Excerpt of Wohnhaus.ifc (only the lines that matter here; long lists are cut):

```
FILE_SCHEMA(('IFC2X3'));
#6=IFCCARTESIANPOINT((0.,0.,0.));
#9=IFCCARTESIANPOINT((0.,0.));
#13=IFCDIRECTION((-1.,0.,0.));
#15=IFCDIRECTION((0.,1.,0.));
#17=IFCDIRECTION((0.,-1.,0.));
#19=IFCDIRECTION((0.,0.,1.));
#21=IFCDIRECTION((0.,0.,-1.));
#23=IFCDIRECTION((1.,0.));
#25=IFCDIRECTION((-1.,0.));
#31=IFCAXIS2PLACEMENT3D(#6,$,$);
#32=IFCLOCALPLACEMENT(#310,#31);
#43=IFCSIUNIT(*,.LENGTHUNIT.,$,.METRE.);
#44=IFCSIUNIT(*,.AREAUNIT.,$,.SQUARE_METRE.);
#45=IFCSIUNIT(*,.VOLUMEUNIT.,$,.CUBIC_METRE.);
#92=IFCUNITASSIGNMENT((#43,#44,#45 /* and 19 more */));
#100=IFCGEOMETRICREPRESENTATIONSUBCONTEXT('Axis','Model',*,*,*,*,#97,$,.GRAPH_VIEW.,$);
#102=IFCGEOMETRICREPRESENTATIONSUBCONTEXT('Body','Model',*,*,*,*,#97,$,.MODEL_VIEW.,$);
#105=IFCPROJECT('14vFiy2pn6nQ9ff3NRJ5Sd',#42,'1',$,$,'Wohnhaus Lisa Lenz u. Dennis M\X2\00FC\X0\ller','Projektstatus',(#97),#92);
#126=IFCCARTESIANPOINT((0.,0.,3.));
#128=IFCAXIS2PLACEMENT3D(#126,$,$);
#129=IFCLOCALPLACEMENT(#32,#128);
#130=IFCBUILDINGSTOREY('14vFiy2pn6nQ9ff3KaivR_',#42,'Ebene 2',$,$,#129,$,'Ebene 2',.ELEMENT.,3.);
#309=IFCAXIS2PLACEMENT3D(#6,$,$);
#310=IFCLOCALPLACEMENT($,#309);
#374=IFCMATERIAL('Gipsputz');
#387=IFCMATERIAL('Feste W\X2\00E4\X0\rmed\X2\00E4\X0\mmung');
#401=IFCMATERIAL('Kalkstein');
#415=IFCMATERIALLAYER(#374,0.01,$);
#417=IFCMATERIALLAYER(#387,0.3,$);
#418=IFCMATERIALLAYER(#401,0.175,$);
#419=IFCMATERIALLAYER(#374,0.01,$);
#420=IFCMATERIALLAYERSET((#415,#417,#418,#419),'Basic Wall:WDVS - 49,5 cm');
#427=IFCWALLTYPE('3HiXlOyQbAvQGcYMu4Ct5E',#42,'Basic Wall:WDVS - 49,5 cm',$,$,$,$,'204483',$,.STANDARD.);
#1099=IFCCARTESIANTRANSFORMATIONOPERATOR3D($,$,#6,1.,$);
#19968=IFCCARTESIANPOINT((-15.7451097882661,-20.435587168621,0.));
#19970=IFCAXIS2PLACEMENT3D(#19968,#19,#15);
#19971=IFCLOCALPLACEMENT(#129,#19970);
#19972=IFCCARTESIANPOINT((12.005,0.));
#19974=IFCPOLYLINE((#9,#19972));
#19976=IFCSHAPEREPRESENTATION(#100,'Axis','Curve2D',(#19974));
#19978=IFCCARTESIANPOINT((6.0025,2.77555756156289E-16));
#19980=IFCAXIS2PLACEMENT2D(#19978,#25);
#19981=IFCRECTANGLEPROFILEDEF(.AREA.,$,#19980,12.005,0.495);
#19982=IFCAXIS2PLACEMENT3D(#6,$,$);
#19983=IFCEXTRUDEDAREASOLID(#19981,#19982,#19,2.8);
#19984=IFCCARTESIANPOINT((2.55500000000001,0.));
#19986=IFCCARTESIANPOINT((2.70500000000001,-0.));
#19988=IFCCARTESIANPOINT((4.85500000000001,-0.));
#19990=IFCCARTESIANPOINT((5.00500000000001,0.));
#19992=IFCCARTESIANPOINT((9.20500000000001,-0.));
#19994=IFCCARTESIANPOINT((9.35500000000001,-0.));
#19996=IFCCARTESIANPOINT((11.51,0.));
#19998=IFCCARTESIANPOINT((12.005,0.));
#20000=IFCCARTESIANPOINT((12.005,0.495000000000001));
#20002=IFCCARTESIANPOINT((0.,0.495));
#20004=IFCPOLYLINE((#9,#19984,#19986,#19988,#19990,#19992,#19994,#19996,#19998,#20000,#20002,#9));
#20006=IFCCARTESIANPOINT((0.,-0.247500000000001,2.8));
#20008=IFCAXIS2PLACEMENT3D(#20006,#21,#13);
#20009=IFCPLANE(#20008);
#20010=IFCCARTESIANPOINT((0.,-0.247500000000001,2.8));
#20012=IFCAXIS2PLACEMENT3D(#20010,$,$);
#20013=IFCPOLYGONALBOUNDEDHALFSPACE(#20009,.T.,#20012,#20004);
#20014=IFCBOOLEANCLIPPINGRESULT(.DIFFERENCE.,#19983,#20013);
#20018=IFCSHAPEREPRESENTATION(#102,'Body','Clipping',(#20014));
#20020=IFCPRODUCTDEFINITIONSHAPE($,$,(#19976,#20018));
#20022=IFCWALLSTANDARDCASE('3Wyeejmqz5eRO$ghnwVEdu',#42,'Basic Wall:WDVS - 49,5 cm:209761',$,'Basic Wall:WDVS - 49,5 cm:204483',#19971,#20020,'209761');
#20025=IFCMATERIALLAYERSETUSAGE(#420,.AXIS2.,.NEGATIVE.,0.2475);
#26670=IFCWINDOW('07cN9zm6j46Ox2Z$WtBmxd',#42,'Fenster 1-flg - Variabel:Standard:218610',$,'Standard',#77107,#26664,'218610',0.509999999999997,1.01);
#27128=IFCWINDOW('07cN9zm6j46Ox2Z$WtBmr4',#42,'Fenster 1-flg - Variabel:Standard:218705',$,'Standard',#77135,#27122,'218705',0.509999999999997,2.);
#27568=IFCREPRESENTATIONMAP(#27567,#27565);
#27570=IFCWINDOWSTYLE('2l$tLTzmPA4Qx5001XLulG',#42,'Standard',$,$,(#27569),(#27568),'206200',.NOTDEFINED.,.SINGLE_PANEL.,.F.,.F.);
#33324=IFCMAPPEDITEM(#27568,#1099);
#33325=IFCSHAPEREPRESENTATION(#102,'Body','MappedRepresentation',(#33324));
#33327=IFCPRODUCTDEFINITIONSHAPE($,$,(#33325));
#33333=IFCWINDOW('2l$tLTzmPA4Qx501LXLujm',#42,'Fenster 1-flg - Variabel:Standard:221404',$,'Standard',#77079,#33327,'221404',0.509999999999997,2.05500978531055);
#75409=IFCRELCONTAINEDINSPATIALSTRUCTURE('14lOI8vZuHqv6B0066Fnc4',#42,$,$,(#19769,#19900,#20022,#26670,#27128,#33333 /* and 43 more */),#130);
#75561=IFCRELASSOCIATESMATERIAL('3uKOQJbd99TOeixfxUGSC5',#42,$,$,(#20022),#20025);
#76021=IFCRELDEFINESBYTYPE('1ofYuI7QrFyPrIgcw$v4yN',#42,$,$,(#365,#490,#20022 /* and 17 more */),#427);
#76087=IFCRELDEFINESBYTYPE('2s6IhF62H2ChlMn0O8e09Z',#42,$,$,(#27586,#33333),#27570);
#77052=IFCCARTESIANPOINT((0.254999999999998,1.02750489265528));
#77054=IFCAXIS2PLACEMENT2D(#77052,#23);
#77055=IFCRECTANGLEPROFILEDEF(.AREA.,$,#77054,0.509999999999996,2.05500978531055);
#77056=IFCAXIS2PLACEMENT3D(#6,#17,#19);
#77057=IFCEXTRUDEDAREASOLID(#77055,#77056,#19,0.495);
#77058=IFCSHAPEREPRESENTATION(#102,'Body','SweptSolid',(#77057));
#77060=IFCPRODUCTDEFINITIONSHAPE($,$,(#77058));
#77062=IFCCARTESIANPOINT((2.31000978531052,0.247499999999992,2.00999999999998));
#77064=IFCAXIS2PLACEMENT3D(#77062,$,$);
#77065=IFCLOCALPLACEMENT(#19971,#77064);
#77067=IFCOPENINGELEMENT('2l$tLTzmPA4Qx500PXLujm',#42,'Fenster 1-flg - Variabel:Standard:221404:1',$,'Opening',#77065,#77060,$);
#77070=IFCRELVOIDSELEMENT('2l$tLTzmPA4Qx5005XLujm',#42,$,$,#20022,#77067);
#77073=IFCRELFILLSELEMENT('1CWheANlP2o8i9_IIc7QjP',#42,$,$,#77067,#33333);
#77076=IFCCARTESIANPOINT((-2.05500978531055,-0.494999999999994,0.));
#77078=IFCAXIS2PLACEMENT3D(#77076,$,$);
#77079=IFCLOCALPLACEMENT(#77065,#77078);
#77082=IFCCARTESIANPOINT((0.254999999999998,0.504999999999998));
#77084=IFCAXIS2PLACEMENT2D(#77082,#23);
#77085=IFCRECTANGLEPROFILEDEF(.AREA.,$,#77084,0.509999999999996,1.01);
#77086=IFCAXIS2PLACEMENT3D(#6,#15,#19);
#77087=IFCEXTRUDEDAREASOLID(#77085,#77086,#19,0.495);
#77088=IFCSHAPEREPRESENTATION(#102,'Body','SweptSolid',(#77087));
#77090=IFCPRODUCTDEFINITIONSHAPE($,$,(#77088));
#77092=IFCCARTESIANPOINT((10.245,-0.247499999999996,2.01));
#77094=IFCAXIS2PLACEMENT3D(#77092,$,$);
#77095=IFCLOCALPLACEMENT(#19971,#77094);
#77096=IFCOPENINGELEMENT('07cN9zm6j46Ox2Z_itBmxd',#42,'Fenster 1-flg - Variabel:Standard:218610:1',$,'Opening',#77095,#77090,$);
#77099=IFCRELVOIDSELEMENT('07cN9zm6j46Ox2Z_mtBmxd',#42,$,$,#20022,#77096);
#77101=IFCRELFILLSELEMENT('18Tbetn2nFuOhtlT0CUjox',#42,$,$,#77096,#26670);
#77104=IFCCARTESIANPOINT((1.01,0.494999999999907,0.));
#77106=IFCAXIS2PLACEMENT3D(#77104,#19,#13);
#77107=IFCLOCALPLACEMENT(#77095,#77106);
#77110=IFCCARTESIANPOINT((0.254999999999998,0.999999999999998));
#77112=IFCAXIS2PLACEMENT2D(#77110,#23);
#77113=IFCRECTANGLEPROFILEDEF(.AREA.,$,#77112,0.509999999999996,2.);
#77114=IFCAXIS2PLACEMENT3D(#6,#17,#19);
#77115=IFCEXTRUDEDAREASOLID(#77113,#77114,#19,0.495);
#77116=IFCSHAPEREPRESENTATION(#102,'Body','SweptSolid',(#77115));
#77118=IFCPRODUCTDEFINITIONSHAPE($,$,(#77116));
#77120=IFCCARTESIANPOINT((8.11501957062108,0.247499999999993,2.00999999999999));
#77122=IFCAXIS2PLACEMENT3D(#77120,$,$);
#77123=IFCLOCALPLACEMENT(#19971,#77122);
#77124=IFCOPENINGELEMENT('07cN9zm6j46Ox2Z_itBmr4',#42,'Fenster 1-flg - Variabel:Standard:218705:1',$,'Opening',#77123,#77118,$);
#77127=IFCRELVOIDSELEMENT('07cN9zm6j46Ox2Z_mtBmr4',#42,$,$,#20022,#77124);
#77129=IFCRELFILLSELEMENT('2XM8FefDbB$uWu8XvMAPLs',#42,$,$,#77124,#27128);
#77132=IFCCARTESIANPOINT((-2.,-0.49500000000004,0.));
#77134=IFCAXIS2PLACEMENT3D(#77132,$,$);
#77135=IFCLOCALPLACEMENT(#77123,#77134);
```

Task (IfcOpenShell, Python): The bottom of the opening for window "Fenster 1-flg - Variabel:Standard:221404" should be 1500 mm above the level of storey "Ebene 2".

```python
import numpy as np
import ifcopenshell
import ifcopenshell.api.geometry
import ifcopenshell.geom
import ifcopenshell.util.element
import ifcopenshell.util.placement
import ifcopenshell.util.shape
import ifcopenshell.util.unit

model = ifcopenshell.open("Wohnhaus.ifc")
unit_scale = ifcopenshell.util.unit.calculate_unit_scale(model)

window = model.by_id(33333)
opening = window.FillsVoids[0].RelatingOpeningElement
storey = ifcopenshell.util.element.get_container(window, ifc_class="IfcBuildingStorey")
level = ifcopenshell.util.placement.get_local_placement(storey.ObjectPlacement)[2, 3]

# The opening's origin need not be at the sill, so measure its lowest point.
shape = ifcopenshell.geom.create_shape(ifcopenshell.geom.settings(), opening)
bottom = ifcopenshell.util.shape.get_shape_bottom_elevation(shape, shape.geometry) / unit_scale
dz = level + 1.5 / unit_scale - bottom

shift = np.array([0.0, 0.0, dz])
# The window is placed relative to its opening, so it follows when the opening moves.
matrix = ifcopenshell.util.placement.get_local_placement(opening.ObjectPlacement)
matrix[:3, 3] += shift
ifcopenshell.api.geometry.edit_object_placement(
    model, product=opening, matrix=matrix, is_si=False, should_transform_children=True
)

print(f"moved by {dz * unit_scale:+.3f} m")

model.write("Wohnhaus_v2.ifc")
```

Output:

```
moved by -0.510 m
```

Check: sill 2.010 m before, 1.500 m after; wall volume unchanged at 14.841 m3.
